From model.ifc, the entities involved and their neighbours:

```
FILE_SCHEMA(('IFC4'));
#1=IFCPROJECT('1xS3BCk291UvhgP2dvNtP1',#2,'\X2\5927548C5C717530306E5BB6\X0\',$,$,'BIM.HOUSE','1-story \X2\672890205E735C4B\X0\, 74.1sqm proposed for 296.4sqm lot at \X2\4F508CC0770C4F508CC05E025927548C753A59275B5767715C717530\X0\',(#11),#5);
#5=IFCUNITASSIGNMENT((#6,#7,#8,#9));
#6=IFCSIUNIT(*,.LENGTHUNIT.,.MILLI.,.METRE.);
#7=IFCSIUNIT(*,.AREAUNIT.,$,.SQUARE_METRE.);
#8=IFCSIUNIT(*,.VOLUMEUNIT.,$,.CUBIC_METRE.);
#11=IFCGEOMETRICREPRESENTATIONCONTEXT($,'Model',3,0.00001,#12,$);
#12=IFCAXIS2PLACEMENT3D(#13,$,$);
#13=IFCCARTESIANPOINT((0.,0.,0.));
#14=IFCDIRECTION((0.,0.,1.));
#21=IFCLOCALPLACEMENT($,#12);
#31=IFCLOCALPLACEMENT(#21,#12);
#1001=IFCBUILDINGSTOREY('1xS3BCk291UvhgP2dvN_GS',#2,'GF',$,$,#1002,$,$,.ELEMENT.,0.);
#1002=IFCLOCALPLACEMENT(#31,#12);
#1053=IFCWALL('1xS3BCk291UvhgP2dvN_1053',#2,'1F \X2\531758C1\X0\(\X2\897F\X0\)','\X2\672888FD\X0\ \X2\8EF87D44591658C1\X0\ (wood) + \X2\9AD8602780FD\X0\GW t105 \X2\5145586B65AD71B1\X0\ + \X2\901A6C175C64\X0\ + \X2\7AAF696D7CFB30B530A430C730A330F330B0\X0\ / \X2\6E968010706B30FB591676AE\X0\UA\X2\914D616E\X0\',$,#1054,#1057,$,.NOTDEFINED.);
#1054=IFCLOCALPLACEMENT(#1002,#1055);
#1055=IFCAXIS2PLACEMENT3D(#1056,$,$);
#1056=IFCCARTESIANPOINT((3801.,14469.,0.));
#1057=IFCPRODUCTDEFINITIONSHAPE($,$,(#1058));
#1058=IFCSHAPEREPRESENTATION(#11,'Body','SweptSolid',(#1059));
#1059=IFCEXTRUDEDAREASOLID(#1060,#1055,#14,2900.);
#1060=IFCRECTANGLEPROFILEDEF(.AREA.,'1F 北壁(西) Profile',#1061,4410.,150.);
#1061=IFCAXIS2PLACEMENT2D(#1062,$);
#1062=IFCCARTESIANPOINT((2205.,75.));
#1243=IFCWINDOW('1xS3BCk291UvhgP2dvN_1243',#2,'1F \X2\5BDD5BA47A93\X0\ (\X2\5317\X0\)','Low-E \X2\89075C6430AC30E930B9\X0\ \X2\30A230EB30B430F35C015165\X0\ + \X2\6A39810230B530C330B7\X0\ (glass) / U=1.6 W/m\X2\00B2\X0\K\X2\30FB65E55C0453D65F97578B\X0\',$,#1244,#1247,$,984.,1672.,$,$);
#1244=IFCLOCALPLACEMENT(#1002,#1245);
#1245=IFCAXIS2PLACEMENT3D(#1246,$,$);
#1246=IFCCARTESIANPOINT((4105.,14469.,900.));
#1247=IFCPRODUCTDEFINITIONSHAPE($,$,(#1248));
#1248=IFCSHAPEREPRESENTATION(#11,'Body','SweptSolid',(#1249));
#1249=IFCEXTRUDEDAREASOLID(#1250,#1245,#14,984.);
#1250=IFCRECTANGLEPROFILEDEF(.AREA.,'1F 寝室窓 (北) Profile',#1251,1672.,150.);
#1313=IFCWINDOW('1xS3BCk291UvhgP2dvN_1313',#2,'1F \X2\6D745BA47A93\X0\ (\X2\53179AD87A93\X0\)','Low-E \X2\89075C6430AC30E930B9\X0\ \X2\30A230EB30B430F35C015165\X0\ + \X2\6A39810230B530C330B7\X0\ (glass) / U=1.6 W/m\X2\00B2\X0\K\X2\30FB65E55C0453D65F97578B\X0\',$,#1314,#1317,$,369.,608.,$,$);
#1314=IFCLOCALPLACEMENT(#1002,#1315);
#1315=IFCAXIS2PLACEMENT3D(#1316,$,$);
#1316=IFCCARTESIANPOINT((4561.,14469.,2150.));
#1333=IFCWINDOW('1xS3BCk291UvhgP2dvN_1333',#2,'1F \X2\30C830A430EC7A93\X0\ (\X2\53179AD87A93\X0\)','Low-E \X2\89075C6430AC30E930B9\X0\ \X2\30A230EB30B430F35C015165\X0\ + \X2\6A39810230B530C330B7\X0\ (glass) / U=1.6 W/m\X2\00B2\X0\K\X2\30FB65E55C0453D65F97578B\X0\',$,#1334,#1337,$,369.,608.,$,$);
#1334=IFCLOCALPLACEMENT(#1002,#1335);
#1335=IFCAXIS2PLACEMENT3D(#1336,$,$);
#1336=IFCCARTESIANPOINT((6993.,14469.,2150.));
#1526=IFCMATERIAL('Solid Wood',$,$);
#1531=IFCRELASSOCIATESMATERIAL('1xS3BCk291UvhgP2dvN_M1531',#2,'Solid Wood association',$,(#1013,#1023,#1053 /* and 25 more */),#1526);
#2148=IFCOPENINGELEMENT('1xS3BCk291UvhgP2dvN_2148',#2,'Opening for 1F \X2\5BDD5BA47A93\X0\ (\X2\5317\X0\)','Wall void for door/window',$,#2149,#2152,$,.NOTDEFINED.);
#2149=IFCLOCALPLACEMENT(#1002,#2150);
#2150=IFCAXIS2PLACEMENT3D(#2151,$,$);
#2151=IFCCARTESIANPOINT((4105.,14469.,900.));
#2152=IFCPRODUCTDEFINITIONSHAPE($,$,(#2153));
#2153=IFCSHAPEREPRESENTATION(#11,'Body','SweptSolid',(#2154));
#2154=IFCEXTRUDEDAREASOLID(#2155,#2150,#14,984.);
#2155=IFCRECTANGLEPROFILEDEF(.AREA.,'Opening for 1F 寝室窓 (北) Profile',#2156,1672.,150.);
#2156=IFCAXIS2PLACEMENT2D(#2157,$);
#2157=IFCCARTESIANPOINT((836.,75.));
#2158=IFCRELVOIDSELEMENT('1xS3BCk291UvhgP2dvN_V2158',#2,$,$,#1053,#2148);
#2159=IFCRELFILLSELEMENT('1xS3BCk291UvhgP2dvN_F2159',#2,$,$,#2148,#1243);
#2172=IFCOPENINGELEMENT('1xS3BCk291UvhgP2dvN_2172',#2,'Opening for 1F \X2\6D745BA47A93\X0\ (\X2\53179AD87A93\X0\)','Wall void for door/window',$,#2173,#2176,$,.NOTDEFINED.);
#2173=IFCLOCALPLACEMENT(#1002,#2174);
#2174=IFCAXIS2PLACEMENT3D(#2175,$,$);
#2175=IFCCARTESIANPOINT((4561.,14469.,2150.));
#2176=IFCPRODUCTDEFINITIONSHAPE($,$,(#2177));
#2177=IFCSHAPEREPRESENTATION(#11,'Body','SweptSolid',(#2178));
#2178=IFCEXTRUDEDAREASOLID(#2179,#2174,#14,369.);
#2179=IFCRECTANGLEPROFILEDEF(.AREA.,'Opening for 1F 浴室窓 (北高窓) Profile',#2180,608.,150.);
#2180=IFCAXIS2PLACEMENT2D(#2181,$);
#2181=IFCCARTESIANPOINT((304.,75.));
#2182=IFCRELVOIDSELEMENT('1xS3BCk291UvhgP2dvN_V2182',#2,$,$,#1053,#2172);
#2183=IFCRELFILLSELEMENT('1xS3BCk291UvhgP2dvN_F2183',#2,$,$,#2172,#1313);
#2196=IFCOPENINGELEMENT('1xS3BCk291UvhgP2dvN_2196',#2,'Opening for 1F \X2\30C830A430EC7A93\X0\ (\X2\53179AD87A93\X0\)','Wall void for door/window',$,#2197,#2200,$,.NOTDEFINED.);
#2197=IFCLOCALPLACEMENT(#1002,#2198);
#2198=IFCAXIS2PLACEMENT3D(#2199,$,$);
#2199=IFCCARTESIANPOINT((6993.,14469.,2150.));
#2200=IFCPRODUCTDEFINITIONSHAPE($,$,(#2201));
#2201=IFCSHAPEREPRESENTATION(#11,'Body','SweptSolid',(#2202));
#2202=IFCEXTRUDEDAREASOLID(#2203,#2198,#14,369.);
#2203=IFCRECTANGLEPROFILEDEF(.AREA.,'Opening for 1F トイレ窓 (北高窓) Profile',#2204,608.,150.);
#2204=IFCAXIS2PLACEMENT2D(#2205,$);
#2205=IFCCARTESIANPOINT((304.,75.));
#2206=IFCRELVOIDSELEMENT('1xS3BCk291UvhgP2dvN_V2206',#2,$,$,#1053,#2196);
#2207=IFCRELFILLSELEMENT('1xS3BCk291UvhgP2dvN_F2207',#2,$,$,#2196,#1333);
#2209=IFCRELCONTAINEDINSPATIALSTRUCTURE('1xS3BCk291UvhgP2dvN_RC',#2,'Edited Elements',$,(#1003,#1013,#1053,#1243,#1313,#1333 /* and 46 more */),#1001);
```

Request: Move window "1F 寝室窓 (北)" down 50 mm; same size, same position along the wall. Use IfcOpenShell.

```python
import numpy as np
import ifcopenshell
import ifcopenshell.api.geometry
import ifcopenshell.util.placement
import ifcopenshell.util.unit

model = ifcopenshell.open("model.ifc")
unit_scale = ifcopenshell.util.unit.calculate_unit_scale(model)

window = model.by_guid("1xS3BCk291UvhgP2dvN_1243")
opening = window.FillsVoids[0].RelatingOpeningElement
dz = -50.0

shift = np.array([0.0, 0.0, dz])
# The window is not placed relative to its opening, so move both.
for product in (opening, window):
    matrix = ifcopenshell.util.placement.get_local_placement(product.ObjectPlacement)
    matrix[:3, 3] += shift
    ifcopenshell.api.geometry.edit_object_placement(model, product=product, matrix=matrix, is_si=False)

print(f"moved by {dz * unit_scale:+.3f} m")

model.write("model_edited.ifc")
```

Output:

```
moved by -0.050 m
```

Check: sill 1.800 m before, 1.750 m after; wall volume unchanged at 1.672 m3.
